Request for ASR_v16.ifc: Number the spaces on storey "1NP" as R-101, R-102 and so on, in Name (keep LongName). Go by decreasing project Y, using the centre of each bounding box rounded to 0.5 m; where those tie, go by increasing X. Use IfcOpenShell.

First a look at what the model holds.

```python
import ifcopenshell
import ifcopenshell.util.element
import ifcopenshell.util.placement

model = ifcopenshell.open("ASR_v16.ifc")
print(model.schema)
storey = next(s for s in model.by_type("IfcBuildingStorey") if s.Name == "1NP")
spaces = [e for e in ifcopenshell.util.element.get_decomposition(storey) if e.is_a("IfcSpace")]
for e in sorted(spaces, key=lambda e: e.id()):
    origin = ifcopenshell.util.placement.get_local_placement(e.ObjectPlacement)[:3, 3]
    print(e.id(), e.Name, e.LongName, origin.round(2) + 0.0, sep=" | ")
```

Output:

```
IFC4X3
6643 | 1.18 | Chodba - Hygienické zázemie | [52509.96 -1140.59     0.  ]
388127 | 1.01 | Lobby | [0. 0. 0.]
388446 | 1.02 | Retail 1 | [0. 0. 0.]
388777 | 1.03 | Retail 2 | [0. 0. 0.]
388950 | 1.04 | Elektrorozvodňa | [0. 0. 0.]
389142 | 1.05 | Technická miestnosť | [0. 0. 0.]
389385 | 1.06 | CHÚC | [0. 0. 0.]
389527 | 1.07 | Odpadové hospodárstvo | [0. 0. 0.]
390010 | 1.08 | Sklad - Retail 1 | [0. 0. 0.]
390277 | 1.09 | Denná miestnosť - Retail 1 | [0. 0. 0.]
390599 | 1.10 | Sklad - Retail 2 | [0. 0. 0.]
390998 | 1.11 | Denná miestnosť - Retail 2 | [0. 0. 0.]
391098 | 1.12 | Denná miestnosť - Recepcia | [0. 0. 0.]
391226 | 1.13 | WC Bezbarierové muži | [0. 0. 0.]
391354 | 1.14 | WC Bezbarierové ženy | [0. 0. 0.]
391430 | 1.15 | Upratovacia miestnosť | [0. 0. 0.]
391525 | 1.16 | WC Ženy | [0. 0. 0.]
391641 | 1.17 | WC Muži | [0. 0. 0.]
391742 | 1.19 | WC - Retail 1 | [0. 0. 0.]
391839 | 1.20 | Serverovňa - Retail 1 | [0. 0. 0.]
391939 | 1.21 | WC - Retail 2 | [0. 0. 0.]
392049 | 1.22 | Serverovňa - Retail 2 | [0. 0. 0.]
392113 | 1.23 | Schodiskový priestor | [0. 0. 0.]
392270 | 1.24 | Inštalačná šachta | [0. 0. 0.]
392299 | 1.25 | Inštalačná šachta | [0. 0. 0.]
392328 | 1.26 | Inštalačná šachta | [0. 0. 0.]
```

```python
import ifcopenshell
import ifcopenshell.geom
import ifcopenshell.util.element
import ifcopenshell.util.shape

model = ifcopenshell.open("ASR_v16.ifc")
settings = ifcopenshell.geom.settings()
settings.set("use-world-coords", True)


def centre(element):
    shape = ifcopenshell.geom.create_shape(settings, element)
    return ifcopenshell.util.shape.get_bbox_centroid(shape.geometry)


storey = next(s for s in model.by_type("IfcBuildingStorey") if s.Name == "1NP")
spaces = [e for e in ifcopenshell.util.element.get_decomposition(storey) if e.is_a("IfcSpace")]

# Insertion points can sit at a corner or the storey origin, so sort by the geometry (in metres).
centres = {e: centre(e) for e in spaces}
spaces.sort(key=lambda e: (-round(centres[e][1] / 0.5), centres[e][0]))

for i, e in enumerate(spaces, start=1):
    number = f"R-1{i:02d}"
    e.Name = number
    print(e.id(), number)

model.write("ASR_v16_edited.ifc")
```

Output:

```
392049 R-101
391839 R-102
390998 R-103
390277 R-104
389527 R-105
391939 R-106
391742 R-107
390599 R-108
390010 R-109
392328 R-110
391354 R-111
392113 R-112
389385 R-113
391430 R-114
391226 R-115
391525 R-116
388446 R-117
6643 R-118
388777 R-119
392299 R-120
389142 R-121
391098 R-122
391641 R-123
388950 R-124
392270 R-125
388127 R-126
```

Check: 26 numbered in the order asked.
